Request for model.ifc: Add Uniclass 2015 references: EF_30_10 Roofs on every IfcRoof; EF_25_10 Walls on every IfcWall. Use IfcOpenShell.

First a look at what the model holds.

```python
import ifcopenshell

model = ifcopenshell.open("model.ifc")
print(model.schema)
print("classifications:", [c.Name for c in model.by_type("IfcClassification")])
for ifc_class in ("IfcDoor", "IfcRoof", "IfcStair", "IfcWall", "IfcWindow"):
    print(ifc_class, len(model.by_type(ifc_class)))
```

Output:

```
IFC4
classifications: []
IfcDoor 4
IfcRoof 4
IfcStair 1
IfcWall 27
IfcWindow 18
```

```python
import ifcopenshell
import ifcopenshell.api.classification

model = ifcopenshell.open("model.ifc")

system = ifcopenshell.api.classification.add_classification(model, classification="Uniclass 2015")

codes = {
    "IfcRoof": ("EF_30_10", "Roofs"),
    "IfcWall": ("EF_25_10", "Walls"),
}
for ifc_class, (code, name) in codes.items():
    products = model.by_type(ifc_class)
    ifcopenshell.api.classification.add_reference(
        model, products=products, classification=system, identification=code, name=name
    )
    print(code, len(products))

model.write("model_v2.ifc")
```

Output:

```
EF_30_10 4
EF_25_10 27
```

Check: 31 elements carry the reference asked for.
